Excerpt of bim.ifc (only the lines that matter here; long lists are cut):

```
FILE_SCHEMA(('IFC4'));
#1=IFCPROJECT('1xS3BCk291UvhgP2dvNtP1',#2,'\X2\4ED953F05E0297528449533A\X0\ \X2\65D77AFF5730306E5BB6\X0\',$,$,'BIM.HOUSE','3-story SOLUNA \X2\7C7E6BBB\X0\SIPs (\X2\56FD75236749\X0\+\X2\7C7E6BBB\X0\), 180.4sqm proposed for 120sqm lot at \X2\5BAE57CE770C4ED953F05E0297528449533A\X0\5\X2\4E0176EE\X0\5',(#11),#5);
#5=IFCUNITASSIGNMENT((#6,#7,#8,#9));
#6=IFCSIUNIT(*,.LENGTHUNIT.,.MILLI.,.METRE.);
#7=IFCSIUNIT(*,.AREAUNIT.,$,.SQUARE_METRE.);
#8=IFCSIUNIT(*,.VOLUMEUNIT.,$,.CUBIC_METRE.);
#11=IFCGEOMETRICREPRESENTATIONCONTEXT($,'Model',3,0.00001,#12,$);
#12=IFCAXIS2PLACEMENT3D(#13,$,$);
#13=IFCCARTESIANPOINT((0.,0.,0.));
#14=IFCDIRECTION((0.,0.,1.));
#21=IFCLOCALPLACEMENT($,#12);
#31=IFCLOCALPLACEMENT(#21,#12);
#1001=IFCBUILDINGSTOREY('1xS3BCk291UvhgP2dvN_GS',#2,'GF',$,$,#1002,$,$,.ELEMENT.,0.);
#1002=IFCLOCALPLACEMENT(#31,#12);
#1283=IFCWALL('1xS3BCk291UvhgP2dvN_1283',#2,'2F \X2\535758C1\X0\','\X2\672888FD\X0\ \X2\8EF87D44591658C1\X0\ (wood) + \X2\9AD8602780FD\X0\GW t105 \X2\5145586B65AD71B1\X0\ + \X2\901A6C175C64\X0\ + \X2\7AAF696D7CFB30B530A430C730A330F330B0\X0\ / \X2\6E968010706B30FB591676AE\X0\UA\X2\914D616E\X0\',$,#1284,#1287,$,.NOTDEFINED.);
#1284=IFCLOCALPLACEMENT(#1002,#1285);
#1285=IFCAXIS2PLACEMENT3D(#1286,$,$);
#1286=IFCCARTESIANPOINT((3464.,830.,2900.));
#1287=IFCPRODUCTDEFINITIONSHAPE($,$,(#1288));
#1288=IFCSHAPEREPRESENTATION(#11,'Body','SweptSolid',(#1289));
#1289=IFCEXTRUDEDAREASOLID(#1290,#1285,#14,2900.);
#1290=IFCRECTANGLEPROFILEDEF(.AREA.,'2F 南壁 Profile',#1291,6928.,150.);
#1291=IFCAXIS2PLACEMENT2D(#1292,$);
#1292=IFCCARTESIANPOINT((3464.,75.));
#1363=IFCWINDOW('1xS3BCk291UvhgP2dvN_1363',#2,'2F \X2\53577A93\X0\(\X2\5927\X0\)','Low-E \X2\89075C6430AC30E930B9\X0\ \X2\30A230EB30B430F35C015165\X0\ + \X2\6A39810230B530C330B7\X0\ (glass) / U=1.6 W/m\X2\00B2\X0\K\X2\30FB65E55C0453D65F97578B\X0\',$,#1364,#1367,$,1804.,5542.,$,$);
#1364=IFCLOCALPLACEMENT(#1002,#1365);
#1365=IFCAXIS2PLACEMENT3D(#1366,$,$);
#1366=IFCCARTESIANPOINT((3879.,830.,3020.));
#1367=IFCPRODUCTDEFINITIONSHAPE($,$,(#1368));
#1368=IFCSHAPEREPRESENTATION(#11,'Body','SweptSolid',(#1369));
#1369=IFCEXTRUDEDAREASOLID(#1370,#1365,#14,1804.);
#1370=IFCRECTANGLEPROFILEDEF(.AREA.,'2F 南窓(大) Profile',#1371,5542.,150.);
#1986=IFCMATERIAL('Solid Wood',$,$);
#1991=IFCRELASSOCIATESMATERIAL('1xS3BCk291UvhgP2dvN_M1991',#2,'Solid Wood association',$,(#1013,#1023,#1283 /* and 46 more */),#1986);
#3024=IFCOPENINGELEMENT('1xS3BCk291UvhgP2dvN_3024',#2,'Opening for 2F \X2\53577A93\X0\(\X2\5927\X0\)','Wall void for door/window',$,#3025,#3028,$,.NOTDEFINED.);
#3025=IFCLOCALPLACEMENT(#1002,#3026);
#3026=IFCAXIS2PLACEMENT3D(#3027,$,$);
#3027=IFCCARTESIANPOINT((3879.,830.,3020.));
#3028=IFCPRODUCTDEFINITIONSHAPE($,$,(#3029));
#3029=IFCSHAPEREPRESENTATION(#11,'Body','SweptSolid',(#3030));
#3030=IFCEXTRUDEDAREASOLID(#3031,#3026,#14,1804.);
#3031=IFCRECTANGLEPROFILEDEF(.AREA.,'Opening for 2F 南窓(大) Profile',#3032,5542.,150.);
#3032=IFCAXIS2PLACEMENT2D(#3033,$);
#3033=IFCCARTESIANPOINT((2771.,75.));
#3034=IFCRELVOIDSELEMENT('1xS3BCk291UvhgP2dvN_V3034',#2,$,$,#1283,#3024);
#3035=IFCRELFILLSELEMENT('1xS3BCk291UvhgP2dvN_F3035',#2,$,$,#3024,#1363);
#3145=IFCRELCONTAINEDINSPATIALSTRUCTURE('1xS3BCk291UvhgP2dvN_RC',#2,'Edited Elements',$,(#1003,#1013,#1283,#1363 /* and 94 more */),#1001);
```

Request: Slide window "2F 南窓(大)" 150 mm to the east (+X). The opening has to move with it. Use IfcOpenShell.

```python
import ifcopenshell
import ifcopenshell.api.geometry
import ifcopenshell.util.placement
import ifcopenshell.util.unit

model = ifcopenshell.open("bim.ifc")
unit_scale = ifcopenshell.util.unit.calculate_unit_scale(model)

window = model.by_guid("1xS3BCk291UvhgP2dvN_1363")
opening = window.FillsVoids[0].RelatingOpeningElement
wall = opening.VoidsElements[0].RelatingBuildingElement

wall_matrix = ifcopenshell.util.placement.get_local_placement(wall.ObjectPlacement)
shift = wall_matrix[:3, 0] * 0.15 / unit_scale
before = ifcopenshell.util.placement.get_local_placement(window.ObjectPlacement)[:3, 3].copy()

# The window is not placed relative to its opening, so move both.
for product in (opening, window):
    matrix = ifcopenshell.util.placement.get_local_placement(product.ObjectPlacement)
    matrix[:3, 3] += shift
    ifcopenshell.api.geometry.edit_object_placement(model, product=product, matrix=matrix, is_si=False)

after = ifcopenshell.util.placement.get_local_placement(window.ObjectPlacement)[:3, 3]
print("window moved by", (after - before).round(3) + 0.0)

model.write("bim_edited.ifc")
```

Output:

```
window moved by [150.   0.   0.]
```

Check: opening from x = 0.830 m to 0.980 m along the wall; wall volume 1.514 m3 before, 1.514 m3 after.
